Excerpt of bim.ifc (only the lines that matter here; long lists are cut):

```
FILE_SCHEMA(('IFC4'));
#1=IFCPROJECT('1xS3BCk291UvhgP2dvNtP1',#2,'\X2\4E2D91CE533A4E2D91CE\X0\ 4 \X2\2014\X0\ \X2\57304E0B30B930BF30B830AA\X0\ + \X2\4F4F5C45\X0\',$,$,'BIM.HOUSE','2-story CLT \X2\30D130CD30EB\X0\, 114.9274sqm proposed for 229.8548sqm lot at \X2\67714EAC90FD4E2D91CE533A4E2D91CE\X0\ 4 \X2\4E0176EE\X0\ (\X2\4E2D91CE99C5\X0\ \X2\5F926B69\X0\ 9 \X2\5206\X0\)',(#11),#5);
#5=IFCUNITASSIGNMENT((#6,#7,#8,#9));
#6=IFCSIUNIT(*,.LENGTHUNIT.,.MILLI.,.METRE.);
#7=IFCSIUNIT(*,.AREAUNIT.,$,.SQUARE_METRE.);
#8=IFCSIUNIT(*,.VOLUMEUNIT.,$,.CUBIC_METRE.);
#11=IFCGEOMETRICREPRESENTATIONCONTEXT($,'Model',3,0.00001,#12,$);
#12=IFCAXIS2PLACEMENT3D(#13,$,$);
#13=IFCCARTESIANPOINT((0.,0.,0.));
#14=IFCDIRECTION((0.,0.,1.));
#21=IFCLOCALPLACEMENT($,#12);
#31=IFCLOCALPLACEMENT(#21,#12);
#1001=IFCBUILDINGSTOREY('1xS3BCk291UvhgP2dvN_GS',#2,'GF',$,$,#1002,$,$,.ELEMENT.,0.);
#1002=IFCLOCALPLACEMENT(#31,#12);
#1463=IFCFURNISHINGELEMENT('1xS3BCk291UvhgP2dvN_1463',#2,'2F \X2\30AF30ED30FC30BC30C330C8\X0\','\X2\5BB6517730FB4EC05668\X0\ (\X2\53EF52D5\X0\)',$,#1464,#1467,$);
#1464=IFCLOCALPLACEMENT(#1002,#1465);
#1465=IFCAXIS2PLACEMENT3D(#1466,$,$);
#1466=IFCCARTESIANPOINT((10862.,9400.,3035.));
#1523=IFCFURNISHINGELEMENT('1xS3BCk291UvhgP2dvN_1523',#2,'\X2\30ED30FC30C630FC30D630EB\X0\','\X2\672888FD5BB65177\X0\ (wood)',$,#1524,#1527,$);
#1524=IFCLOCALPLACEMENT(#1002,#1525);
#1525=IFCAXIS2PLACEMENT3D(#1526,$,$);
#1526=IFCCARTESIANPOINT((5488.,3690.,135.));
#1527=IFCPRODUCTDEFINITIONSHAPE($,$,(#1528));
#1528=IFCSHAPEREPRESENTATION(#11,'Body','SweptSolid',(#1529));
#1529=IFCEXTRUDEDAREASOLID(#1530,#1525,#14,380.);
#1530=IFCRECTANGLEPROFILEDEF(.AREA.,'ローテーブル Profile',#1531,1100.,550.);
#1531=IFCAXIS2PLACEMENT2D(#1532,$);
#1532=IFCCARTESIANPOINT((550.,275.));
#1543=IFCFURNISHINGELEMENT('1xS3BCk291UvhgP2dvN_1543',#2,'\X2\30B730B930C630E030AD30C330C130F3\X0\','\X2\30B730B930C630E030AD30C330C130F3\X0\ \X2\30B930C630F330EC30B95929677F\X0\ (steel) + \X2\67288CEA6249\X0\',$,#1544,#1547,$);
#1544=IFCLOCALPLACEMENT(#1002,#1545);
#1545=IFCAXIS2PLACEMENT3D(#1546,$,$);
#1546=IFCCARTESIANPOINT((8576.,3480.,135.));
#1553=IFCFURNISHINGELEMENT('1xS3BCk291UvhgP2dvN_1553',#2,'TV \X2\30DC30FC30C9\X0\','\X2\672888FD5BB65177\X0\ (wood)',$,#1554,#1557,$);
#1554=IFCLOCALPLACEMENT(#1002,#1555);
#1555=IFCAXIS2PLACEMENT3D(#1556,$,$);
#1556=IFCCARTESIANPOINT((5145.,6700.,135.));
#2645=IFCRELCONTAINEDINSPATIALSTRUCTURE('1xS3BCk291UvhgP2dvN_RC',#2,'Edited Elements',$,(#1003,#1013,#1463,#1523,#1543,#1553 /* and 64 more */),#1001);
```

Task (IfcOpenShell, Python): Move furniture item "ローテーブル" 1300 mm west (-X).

```python
import ifcopenshell
import ifcopenshell.api.geometry
import ifcopenshell.util.placement

model = ifcopenshell.open("bim.ifc")

item = model.by_guid("1xS3BCk291UvhgP2dvN_1523")
matrix = ifcopenshell.util.placement.get_local_placement(item.ObjectPlacement)
matrix[0, 3] -= 1300.0
ifcopenshell.api.geometry.edit_object_placement(model, product=item, matrix=matrix, is_si=False)

print(ifcopenshell.util.placement.get_local_placement(item.ObjectPlacement).round(3) + 0.0)

model.write("bim_edited.ifc")
```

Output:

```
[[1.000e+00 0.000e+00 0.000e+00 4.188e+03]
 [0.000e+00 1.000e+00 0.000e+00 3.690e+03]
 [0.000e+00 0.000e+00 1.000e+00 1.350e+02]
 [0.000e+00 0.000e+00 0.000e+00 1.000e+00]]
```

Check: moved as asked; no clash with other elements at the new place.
